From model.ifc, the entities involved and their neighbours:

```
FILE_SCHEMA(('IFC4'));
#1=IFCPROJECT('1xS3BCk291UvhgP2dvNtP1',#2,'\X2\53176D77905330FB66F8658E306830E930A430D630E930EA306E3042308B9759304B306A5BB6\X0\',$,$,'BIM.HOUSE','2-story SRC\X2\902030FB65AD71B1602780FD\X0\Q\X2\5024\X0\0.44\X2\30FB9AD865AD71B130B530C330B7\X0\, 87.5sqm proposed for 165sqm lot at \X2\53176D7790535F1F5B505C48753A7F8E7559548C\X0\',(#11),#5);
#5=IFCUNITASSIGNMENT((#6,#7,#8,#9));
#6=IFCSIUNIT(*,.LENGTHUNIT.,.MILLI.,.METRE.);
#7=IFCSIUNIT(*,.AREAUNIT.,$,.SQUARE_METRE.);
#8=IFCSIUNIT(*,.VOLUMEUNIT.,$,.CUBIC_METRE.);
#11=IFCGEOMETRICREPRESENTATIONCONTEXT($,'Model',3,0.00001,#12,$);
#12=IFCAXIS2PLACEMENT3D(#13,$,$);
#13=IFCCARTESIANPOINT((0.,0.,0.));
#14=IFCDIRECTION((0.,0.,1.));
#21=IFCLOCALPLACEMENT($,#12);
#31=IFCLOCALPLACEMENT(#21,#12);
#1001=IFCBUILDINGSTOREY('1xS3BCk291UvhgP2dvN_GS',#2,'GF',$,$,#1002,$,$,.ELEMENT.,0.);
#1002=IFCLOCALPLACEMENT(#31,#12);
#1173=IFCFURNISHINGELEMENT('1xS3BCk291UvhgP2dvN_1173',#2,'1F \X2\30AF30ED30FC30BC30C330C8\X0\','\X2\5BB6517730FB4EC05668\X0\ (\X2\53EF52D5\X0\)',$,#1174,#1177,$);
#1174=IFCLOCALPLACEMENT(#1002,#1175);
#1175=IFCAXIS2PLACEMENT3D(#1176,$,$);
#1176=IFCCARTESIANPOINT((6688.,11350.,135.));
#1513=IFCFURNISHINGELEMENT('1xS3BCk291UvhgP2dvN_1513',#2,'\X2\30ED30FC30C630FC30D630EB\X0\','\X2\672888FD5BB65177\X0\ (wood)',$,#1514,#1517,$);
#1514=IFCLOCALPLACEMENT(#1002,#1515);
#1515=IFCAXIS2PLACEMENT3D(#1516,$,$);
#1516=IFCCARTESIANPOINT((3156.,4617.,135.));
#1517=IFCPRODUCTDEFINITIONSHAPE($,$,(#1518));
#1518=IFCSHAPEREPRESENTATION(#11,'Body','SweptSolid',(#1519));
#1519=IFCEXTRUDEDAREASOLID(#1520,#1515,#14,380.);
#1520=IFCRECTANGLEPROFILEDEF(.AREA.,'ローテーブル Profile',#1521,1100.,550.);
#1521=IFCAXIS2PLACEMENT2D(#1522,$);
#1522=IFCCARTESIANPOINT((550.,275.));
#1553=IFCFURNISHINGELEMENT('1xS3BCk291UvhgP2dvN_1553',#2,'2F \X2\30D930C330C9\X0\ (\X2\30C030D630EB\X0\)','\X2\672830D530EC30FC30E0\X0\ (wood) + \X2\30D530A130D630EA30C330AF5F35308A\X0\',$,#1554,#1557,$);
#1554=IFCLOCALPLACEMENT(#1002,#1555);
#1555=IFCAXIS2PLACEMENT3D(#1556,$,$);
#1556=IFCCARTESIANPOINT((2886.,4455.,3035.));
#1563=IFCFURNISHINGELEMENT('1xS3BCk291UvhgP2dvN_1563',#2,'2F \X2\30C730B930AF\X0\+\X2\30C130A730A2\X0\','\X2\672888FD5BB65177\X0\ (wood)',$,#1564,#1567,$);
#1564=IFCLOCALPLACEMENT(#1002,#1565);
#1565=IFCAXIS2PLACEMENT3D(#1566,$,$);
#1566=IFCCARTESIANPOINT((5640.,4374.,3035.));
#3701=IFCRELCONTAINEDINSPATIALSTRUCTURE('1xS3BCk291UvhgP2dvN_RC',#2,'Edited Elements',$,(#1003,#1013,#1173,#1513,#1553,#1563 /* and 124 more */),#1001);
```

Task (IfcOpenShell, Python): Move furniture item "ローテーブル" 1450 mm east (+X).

```python
import ifcopenshell
import ifcopenshell.api.geometry
import ifcopenshell.util.placement
import ifcopenshell.util.unit

model = ifcopenshell.open("model.ifc")
unit_scale = ifcopenshell.util.unit.calculate_unit_scale(model)

item = model.by_id(1513)
matrix = ifcopenshell.util.placement.get_local_placement(item.ObjectPlacement)
matrix[0, 3] += 1.45 / unit_scale
ifcopenshell.api.geometry.edit_object_placement(model, product=item, matrix=matrix, is_si=False)

print(ifcopenshell.util.placement.get_local_placement(item.ObjectPlacement).round(3) + 0.0)

model.write("model-out.ifc")
```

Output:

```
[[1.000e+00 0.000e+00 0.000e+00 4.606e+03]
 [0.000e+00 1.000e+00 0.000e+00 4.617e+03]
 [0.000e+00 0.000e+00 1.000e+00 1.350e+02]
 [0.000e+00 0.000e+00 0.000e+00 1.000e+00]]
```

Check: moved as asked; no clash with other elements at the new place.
